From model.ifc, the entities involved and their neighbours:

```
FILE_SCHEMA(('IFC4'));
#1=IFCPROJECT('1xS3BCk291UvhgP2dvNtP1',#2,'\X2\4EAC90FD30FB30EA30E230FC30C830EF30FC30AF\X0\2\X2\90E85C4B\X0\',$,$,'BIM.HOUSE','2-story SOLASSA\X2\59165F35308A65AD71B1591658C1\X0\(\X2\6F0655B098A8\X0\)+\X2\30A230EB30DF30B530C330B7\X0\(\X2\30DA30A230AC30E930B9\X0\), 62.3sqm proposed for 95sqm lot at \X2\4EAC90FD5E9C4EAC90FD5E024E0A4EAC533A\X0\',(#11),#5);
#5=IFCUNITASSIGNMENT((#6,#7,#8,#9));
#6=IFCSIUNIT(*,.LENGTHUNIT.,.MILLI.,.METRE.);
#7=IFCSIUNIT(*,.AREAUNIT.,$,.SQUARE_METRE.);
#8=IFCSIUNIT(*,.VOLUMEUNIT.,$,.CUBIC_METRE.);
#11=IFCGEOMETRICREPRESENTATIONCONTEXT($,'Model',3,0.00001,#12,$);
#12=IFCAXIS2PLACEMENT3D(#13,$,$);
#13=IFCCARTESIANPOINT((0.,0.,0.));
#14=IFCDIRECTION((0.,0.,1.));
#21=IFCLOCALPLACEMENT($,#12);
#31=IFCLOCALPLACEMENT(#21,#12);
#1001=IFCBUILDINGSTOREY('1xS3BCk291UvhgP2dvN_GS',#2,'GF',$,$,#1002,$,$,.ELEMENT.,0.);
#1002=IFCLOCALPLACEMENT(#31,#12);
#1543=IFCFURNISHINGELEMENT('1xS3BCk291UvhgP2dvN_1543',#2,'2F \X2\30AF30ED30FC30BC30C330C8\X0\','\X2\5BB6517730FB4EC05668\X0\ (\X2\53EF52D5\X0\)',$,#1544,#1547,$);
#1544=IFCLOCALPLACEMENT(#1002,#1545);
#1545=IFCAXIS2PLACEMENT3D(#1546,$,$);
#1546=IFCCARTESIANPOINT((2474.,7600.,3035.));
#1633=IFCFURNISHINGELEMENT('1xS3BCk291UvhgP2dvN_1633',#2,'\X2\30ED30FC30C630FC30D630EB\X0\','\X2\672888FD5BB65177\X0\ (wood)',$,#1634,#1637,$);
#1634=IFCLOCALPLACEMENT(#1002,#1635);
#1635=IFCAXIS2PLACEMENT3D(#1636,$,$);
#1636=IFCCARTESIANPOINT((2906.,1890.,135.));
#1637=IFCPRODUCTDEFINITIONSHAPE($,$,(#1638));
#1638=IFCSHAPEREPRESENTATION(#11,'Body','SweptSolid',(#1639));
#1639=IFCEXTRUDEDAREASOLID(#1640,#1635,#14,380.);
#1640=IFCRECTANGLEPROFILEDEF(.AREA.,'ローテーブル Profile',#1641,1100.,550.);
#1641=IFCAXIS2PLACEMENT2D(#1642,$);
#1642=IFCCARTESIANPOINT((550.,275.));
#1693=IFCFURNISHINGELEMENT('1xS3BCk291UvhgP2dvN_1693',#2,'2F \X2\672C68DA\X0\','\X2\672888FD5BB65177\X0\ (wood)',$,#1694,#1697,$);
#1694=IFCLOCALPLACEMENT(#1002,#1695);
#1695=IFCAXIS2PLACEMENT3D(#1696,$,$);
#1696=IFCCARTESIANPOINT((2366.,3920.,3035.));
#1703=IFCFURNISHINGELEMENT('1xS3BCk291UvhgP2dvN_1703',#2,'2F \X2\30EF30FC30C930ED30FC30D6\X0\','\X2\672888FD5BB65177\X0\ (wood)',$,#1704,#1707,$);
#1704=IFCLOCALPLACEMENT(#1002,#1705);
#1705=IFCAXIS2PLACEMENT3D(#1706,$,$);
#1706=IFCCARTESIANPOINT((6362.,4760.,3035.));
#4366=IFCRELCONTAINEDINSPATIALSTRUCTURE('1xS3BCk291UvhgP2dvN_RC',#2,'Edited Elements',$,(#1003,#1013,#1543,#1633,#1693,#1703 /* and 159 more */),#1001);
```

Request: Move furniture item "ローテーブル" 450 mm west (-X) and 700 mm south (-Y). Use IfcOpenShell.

```python
import ifcopenshell
import ifcopenshell.api.geometry
import ifcopenshell.util.placement
import ifcopenshell.util.unit

model = ifcopenshell.open("model.ifc")
unit_scale = ifcopenshell.util.unit.calculate_unit_scale(model)

item = model.by_guid("1xS3BCk291UvhgP2dvN_1633")
matrix = ifcopenshell.util.placement.get_local_placement(item.ObjectPlacement)
matrix[0, 3] -= 0.45 / unit_scale
matrix[1, 3] -= 0.7 / unit_scale
ifcopenshell.api.geometry.edit_object_placement(model, product=item, matrix=matrix, is_si=False)

print(ifcopenshell.util.placement.get_local_placement(item.ObjectPlacement).round(3) + 0.0)

model.write("model_edited.ifc")
```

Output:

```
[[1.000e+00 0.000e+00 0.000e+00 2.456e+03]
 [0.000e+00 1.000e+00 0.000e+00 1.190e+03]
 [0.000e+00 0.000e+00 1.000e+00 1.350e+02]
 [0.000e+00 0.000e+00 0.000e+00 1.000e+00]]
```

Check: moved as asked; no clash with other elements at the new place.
